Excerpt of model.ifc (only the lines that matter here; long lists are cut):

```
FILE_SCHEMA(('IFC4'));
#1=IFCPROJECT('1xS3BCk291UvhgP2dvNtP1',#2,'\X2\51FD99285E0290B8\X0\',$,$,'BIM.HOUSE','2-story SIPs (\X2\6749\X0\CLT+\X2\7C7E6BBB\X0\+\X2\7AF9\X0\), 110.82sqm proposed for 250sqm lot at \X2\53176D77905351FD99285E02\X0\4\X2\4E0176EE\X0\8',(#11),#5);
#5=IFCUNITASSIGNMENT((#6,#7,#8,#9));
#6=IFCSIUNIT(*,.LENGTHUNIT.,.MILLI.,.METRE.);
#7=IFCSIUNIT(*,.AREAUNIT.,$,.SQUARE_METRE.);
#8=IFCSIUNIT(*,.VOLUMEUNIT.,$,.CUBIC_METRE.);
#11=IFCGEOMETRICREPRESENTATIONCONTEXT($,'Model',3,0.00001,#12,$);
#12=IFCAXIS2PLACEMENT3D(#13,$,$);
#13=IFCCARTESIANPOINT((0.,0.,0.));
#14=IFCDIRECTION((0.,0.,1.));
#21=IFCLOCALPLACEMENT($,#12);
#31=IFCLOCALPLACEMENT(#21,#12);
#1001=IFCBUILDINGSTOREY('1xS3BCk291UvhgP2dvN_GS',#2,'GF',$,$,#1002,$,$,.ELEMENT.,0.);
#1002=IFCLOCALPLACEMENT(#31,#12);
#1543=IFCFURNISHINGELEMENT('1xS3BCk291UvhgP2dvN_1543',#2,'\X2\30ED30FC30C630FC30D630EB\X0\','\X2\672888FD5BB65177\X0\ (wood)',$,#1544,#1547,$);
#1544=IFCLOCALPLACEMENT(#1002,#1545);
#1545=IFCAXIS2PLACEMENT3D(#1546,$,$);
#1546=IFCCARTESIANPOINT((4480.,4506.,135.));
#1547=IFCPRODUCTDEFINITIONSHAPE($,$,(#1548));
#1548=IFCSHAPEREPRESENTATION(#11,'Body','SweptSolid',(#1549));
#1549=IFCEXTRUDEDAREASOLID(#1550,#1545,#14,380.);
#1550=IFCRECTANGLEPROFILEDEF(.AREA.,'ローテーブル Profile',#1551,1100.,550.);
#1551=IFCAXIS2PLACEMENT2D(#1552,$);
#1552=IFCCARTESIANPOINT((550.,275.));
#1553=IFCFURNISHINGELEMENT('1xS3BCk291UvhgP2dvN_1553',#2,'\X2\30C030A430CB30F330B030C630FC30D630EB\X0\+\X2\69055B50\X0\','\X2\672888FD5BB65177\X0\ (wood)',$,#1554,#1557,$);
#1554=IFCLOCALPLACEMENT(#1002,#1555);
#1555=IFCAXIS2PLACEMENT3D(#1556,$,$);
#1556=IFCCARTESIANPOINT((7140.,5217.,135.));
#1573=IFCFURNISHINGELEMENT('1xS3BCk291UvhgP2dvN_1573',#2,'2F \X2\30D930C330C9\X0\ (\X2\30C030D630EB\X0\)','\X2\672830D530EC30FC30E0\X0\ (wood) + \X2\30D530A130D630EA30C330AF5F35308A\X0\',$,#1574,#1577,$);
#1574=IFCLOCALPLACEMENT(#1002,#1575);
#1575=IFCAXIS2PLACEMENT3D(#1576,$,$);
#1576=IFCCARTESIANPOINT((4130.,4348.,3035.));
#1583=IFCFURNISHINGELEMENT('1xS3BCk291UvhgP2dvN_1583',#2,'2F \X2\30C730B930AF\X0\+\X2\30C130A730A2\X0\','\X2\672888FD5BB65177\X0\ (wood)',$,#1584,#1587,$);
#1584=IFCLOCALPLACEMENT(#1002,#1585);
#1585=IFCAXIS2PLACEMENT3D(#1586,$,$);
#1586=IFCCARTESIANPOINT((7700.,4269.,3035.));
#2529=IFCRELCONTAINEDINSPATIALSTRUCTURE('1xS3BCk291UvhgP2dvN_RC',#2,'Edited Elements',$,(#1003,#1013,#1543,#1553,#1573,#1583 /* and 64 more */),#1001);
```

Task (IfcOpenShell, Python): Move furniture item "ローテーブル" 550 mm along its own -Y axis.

```python
import ifcopenshell
import ifcopenshell.api.geometry
import ifcopenshell.util.placement

model = ifcopenshell.open("model.ifc")

item = model.by_guid("1xS3BCk291UvhgP2dvN_1543")
matrix = ifcopenshell.util.placement.get_local_placement(item.ObjectPlacement)
matrix[:3, 3] -= matrix[:3, 1] * 550.0
ifcopenshell.api.geometry.edit_object_placement(model, product=item, matrix=matrix, is_si=False)

print(ifcopenshell.util.placement.get_local_placement(item.ObjectPlacement).round(3) + 0.0)

model.write("model_v2.ifc")
```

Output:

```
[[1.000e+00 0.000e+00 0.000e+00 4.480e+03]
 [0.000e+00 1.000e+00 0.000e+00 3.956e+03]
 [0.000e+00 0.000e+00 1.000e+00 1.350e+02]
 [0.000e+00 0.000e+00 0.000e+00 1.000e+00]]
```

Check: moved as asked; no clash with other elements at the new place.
